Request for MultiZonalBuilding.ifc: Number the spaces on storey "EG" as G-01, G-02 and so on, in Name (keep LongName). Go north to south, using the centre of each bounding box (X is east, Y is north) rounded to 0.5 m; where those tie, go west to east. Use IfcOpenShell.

First a look at what the model holds.

```python
import ifcopenshell
import ifcopenshell.util.element
import ifcopenshell.util.placement

model = ifcopenshell.open("MultiZonalBuilding.ifc")
print(model.schema)
storey = next(s for s in model.by_type("IfcBuildingStorey") if s.Name == "EG")
spaces = [e for e in ifcopenshell.util.element.get_decomposition(storey) if e.is_a("IfcSpace")]
for e in sorted(spaces, key=lambda e: e.id()):
    origin = ifcopenshell.util.placement.get_local_placement(e.ObjectPlacement)[:3, 3]
    print(e.id(), e.Name, e.LongName, origin.round(2) + 0.0, sep=" | ")
```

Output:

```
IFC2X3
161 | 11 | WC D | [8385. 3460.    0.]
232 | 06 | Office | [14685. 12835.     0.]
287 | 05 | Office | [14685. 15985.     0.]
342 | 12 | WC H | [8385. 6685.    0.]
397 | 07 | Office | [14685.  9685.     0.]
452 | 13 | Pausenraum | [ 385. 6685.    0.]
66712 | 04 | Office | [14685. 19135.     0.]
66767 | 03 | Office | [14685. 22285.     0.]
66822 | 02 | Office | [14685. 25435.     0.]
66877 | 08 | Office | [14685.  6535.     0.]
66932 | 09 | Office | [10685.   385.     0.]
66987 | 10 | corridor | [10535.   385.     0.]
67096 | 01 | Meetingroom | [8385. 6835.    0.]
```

```python
import ifcopenshell
import ifcopenshell.geom
import ifcopenshell.util.element
import ifcopenshell.util.shape

model = ifcopenshell.open("MultiZonalBuilding.ifc")
settings = ifcopenshell.geom.settings()
settings.set("use-world-coords", True)


def centre(element):
    shape = ifcopenshell.geom.create_shape(settings, element)
    return ifcopenshell.util.shape.get_bbox_centroid(shape.geometry)


storey = next(s for s in model.by_type("IfcBuildingStorey") if s.Name == "EG")
spaces = [e for e in ifcopenshell.util.element.get_decomposition(storey) if e.is_a("IfcSpace")]

# Insertion points can sit at a corner or the storey origin, so sort by the geometry (in metres).
centres = {e: centre(e) for e in spaces}
spaces.sort(key=lambda e: (-round(centres[e][1] / 0.5), centres[e][0]))

for i, e in enumerate(spaces, start=1):
    number = f"G-{i:02d}"
    e.Name = number
    print(e.id(), number)

model.write("MultiZonalBuilding_updated.ifc")
```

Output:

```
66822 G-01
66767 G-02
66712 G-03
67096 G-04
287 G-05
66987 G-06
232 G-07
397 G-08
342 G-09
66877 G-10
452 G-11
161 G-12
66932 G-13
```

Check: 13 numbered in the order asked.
